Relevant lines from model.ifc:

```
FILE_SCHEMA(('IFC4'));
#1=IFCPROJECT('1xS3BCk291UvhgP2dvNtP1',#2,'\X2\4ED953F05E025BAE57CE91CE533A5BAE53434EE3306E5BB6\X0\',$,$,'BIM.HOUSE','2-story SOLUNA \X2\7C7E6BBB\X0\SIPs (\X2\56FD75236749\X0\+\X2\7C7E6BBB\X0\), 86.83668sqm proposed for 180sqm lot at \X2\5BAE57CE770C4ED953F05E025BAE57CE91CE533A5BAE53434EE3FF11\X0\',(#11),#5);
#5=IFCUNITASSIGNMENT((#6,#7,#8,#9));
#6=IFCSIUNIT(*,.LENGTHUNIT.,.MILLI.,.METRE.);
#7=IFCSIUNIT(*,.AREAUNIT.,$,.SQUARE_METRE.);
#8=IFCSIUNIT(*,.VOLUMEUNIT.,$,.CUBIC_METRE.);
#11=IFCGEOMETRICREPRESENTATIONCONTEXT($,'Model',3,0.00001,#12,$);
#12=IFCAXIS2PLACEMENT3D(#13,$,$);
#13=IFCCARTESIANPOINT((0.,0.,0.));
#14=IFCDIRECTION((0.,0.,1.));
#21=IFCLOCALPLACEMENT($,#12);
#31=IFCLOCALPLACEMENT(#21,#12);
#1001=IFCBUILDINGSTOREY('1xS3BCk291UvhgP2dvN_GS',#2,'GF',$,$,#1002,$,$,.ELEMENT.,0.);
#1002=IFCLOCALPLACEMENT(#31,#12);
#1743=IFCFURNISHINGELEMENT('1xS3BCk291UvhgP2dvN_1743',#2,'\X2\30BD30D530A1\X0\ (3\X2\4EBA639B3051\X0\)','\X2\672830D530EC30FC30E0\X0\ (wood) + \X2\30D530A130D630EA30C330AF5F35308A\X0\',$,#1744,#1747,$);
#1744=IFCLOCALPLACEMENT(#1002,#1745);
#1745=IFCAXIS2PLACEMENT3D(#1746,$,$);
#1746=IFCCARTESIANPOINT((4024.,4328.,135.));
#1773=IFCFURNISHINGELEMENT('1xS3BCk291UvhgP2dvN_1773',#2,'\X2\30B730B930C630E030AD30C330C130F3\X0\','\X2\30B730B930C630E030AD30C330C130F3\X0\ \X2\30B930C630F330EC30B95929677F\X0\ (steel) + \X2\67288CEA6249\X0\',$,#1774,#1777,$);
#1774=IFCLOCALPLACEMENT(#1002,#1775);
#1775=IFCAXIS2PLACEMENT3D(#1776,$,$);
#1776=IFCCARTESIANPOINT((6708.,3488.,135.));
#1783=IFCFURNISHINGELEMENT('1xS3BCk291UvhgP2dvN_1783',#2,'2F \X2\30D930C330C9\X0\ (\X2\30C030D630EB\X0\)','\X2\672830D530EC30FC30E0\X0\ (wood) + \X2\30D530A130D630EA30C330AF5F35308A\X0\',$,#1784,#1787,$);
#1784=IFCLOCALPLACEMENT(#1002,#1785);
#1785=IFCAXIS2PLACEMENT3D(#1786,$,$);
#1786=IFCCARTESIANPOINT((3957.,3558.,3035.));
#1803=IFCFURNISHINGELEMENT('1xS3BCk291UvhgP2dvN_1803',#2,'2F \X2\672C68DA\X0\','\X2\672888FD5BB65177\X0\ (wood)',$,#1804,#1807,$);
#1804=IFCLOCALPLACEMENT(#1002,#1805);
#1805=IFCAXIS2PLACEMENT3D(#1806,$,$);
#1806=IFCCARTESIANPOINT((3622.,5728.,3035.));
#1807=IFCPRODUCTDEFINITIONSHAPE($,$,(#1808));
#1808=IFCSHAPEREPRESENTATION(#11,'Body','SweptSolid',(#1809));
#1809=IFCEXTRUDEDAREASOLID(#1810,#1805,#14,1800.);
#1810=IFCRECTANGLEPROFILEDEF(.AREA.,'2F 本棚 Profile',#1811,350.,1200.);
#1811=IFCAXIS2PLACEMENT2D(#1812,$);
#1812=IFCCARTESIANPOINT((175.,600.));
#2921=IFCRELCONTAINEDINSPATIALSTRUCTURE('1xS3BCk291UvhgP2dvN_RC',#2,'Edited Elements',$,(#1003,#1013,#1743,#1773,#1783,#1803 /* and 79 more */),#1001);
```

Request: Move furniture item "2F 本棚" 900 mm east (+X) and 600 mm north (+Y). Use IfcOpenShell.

```python
import ifcopenshell
import ifcopenshell.api.geometry
import ifcopenshell.util.placement
import ifcopenshell.util.unit

model = ifcopenshell.open("model.ifc")
unit_scale = ifcopenshell.util.unit.calculate_unit_scale(model)

item = model.by_guid("1xS3BCk291UvhgP2dvN_1803")
matrix = ifcopenshell.util.placement.get_local_placement(item.ObjectPlacement)
matrix[0, 3] += 0.9 / unit_scale
matrix[1, 3] += 0.6 / unit_scale
ifcopenshell.api.geometry.edit_object_placement(model, product=item, matrix=matrix, is_si=False)

print(ifcopenshell.util.placement.get_local_placement(item.ObjectPlacement).round(3) + 0.0)

model.write("model_updated.ifc")
```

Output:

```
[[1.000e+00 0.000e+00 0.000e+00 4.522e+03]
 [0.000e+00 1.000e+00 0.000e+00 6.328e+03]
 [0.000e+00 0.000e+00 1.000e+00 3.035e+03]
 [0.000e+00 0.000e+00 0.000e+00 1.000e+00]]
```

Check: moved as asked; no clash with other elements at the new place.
